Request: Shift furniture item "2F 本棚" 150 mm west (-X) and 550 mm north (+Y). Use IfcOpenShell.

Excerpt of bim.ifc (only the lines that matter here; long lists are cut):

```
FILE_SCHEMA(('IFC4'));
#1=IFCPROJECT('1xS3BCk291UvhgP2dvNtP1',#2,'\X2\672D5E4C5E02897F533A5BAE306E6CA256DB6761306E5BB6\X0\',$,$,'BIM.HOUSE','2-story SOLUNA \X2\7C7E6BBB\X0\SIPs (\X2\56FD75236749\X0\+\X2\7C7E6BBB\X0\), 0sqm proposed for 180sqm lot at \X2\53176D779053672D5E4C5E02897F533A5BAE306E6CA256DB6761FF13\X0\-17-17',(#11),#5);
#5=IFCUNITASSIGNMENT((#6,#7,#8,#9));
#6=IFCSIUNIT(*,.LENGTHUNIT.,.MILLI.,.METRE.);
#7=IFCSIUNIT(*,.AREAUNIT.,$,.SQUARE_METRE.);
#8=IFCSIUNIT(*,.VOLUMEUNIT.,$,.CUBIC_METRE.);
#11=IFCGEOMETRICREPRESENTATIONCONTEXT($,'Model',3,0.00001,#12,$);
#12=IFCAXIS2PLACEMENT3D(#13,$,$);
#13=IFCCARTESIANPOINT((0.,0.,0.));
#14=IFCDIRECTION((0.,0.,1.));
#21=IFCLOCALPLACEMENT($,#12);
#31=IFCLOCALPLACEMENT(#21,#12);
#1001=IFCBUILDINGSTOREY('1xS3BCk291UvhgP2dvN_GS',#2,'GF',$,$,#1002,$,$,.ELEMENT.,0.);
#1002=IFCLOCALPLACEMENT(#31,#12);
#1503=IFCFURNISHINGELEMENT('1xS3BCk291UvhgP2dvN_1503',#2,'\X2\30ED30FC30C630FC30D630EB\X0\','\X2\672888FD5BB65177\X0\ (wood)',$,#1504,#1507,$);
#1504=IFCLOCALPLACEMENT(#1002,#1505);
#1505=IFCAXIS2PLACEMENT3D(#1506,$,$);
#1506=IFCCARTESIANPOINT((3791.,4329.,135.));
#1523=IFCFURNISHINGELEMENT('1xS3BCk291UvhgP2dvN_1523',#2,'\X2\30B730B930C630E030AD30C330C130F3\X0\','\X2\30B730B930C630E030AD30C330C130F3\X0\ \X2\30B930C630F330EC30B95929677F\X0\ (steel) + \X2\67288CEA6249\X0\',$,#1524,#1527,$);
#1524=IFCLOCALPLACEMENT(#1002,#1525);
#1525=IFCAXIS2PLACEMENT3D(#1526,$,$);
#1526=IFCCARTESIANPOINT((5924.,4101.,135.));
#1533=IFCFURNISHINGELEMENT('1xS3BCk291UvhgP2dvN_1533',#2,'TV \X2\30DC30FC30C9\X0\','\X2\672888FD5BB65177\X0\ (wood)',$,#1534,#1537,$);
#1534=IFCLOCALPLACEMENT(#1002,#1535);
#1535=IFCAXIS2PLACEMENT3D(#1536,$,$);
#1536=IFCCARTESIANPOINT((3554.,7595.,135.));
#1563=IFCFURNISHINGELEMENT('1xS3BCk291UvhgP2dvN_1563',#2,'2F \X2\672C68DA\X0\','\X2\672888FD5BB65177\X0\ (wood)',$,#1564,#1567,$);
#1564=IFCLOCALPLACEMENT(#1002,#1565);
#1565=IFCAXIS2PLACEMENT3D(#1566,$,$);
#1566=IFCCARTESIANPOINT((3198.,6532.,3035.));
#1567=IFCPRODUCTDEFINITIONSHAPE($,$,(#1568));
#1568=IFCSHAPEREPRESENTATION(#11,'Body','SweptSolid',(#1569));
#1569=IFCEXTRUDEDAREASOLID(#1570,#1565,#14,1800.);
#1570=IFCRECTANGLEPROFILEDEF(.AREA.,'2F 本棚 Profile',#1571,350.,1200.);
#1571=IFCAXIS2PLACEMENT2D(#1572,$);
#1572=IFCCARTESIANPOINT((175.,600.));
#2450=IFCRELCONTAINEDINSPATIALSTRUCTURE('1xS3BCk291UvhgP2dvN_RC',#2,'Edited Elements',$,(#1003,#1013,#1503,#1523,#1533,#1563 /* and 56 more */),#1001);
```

```python
import ifcopenshell
import ifcopenshell.api.geometry
import ifcopenshell.util.placement

model = ifcopenshell.open("bim.ifc")

item = model.by_id(1563)
matrix = ifcopenshell.util.placement.get_local_placement(item.ObjectPlacement)
matrix[0, 3] -= 150.0
matrix[1, 3] += 550.0
ifcopenshell.api.geometry.edit_object_placement(model, product=item, matrix=matrix, is_si=False)

print(ifcopenshell.util.placement.get_local_placement(item.ObjectPlacement).round(3) + 0.0)

model.write("bim_edited.ifc")
```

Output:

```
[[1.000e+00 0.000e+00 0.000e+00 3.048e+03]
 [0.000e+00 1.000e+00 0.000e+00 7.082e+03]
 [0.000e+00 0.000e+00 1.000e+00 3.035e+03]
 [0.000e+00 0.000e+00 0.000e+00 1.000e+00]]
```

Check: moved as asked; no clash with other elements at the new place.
